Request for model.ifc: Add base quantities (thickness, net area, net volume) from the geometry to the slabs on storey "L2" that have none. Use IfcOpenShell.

First a look at what the model holds.

```python
import ifcopenshell
import ifcopenshell.util.element
import ifcopenshell.util.unit

model = ifcopenshell.open("model.ifc")
print(model.schema)
for unit_type in ("LENGTHUNIT", "AREAUNIT", "VOLUMEUNIT"):
    print(unit_type, ifcopenshell.util.unit.calculate_unit_scale(model, unit_type))
storey = next(s for s in model.by_type("IfcBuildingStorey") if s.Name == "L2")
slabs = [e for e in ifcopenshell.util.element.get_decomposition(storey) if e.is_a("IfcSlab")]
for e in sorted(slabs, key=lambda e: e.id()):
    print(e.id(), e.is_a(), e.Name, list(ifcopenshell.util.element.get_psets(e, qtos_only=True)), sep=" | ")
```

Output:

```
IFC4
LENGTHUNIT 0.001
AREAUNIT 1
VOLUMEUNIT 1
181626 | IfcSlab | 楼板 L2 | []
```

```python
import ifcopenshell
import ifcopenshell.api.pset
import ifcopenshell.geom
import ifcopenshell.util.element
import ifcopenshell.util.shape
import ifcopenshell.util.unit

model = ifcopenshell.open("model.ifc")
unit_scale = ifcopenshell.util.unit.calculate_unit_scale(model)
area_scale = ifcopenshell.util.unit.calculate_unit_scale(model, "AREAUNIT")
volume_scale = ifcopenshell.util.unit.calculate_unit_scale(model, "VOLUMEUNIT")
settings = ifcopenshell.geom.settings()

storey = next(s for s in model.by_type("IfcBuildingStorey") if s.Name == "L2")
slabs = [e for e in ifcopenshell.util.element.get_decomposition(storey) if e.is_a("IfcSlab")]

for e in sorted(slabs, key=lambda e: e.id()):
    if ifcopenshell.util.element.get_psets(e, qtos_only=True, should_inherit=False):
        continue
    # Geometry comes back in metres, in the element's own axes.
    shape = ifcopenshell.geom.create_shape(settings, e)
    values = {
        "Width": ifcopenshell.util.shape.get_z(shape.geometry) / unit_scale,
        "NetArea": ifcopenshell.util.shape.get_footprint_area(shape.geometry) / area_scale,
        "NetVolume": ifcopenshell.util.shape.get_volume(shape.geometry) / volume_scale,
    }
    qto = ifcopenshell.api.pset.add_qto(model, product=e, name="Qto_SlabBaseQuantities")
    ifcopenshell.api.pset.edit_qto(model, qto=qto, properties=values)
    print(e.id(), {k: round(v, 3) for k, v in values.items()})

model.write("model_updated.ifc")
```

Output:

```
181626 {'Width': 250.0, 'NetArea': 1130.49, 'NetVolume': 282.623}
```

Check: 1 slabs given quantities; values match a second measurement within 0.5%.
